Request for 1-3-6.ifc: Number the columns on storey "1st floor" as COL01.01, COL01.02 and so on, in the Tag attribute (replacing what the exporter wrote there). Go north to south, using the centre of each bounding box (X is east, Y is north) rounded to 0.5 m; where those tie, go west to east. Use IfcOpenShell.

First a look at what the model holds.

```python
import ifcopenshell
import ifcopenshell.util.element
import ifcopenshell.util.placement

model = ifcopenshell.open("1-3-6.ifc")
print(model.schema)
storey = next(s for s in model.by_type("IfcBuildingStorey") if s.Name == "1st floor")
columns = [e for e in ifcopenshell.util.element.get_decomposition(storey) if e.is_a("IfcColumn")]
for e in sorted(columns, key=lambda e: e.id()):
    origin = ifcopenshell.util.placement.get_local_placement(e.ObjectPlacement)[:3, 3]
    print(e.id(), e.Tag, e.Name, origin.round(2) + 0.0, sep=" | ")
```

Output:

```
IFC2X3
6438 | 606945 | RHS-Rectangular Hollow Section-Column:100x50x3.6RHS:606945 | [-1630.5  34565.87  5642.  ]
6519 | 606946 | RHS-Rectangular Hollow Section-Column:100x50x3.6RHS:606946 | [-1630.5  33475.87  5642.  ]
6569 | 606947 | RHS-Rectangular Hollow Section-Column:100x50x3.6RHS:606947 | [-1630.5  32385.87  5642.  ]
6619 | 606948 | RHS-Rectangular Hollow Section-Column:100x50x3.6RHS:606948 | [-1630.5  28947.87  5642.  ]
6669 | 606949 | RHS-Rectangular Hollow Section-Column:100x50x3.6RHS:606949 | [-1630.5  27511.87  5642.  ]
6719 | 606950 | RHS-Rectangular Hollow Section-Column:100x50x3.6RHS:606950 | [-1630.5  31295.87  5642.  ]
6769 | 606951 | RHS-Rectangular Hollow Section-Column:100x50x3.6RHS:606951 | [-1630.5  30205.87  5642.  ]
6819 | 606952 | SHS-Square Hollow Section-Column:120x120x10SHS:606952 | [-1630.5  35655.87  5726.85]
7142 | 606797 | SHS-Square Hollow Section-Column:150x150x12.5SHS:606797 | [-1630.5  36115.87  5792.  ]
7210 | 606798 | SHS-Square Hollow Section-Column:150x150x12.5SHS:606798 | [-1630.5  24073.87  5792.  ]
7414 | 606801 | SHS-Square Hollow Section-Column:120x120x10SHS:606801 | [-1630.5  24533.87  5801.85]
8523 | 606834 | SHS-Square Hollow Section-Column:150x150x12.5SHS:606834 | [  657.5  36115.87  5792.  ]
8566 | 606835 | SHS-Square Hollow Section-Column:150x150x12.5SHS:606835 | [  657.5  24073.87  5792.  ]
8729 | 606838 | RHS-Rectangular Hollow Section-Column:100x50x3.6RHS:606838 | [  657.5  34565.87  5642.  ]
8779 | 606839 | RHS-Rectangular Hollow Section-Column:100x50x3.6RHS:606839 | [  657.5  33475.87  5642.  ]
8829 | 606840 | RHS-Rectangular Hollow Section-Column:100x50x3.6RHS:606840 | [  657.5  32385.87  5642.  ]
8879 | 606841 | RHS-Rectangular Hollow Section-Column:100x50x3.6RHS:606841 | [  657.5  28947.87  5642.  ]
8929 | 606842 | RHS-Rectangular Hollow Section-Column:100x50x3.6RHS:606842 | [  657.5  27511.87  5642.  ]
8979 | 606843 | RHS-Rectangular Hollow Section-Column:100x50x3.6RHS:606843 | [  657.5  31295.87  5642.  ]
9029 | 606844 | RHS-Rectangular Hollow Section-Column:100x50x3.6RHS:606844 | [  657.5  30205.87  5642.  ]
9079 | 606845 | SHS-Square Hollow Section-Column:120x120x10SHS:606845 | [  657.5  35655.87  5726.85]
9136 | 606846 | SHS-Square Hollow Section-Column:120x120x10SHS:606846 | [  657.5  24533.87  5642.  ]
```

```python
import ifcopenshell
import ifcopenshell.geom
import ifcopenshell.util.element
import ifcopenshell.util.shape

model = ifcopenshell.open("1-3-6.ifc")
settings = ifcopenshell.geom.settings()
settings.set("use-world-coords", True)


def centre(element):
    shape = ifcopenshell.geom.create_shape(settings, element)
    return ifcopenshell.util.shape.get_bbox_centroid(shape.geometry)


storey = next(s for s in model.by_type("IfcBuildingStorey") if s.Name == "1st floor")
columns = [e for e in ifcopenshell.util.element.get_decomposition(storey) if e.is_a("IfcColumn")]

# Insertion points can sit at a corner or the storey origin, so sort by the geometry (in metres).
centres = {e: centre(e) for e in columns}
columns.sort(key=lambda e: (-round(centres[e][1] / 0.5), centres[e][0]))

for i, e in enumerate(columns, start=1):
    number = f"COL01.{i:02d}"
    e.Tag = number
    print(e.id(), number)

model.write("1-3-6_updated.ifc")
```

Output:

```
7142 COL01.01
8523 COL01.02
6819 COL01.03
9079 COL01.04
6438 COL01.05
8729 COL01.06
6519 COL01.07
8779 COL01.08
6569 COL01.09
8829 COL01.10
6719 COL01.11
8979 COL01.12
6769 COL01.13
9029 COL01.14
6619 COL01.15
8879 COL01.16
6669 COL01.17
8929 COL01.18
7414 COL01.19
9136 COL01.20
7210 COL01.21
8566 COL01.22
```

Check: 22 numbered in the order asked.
